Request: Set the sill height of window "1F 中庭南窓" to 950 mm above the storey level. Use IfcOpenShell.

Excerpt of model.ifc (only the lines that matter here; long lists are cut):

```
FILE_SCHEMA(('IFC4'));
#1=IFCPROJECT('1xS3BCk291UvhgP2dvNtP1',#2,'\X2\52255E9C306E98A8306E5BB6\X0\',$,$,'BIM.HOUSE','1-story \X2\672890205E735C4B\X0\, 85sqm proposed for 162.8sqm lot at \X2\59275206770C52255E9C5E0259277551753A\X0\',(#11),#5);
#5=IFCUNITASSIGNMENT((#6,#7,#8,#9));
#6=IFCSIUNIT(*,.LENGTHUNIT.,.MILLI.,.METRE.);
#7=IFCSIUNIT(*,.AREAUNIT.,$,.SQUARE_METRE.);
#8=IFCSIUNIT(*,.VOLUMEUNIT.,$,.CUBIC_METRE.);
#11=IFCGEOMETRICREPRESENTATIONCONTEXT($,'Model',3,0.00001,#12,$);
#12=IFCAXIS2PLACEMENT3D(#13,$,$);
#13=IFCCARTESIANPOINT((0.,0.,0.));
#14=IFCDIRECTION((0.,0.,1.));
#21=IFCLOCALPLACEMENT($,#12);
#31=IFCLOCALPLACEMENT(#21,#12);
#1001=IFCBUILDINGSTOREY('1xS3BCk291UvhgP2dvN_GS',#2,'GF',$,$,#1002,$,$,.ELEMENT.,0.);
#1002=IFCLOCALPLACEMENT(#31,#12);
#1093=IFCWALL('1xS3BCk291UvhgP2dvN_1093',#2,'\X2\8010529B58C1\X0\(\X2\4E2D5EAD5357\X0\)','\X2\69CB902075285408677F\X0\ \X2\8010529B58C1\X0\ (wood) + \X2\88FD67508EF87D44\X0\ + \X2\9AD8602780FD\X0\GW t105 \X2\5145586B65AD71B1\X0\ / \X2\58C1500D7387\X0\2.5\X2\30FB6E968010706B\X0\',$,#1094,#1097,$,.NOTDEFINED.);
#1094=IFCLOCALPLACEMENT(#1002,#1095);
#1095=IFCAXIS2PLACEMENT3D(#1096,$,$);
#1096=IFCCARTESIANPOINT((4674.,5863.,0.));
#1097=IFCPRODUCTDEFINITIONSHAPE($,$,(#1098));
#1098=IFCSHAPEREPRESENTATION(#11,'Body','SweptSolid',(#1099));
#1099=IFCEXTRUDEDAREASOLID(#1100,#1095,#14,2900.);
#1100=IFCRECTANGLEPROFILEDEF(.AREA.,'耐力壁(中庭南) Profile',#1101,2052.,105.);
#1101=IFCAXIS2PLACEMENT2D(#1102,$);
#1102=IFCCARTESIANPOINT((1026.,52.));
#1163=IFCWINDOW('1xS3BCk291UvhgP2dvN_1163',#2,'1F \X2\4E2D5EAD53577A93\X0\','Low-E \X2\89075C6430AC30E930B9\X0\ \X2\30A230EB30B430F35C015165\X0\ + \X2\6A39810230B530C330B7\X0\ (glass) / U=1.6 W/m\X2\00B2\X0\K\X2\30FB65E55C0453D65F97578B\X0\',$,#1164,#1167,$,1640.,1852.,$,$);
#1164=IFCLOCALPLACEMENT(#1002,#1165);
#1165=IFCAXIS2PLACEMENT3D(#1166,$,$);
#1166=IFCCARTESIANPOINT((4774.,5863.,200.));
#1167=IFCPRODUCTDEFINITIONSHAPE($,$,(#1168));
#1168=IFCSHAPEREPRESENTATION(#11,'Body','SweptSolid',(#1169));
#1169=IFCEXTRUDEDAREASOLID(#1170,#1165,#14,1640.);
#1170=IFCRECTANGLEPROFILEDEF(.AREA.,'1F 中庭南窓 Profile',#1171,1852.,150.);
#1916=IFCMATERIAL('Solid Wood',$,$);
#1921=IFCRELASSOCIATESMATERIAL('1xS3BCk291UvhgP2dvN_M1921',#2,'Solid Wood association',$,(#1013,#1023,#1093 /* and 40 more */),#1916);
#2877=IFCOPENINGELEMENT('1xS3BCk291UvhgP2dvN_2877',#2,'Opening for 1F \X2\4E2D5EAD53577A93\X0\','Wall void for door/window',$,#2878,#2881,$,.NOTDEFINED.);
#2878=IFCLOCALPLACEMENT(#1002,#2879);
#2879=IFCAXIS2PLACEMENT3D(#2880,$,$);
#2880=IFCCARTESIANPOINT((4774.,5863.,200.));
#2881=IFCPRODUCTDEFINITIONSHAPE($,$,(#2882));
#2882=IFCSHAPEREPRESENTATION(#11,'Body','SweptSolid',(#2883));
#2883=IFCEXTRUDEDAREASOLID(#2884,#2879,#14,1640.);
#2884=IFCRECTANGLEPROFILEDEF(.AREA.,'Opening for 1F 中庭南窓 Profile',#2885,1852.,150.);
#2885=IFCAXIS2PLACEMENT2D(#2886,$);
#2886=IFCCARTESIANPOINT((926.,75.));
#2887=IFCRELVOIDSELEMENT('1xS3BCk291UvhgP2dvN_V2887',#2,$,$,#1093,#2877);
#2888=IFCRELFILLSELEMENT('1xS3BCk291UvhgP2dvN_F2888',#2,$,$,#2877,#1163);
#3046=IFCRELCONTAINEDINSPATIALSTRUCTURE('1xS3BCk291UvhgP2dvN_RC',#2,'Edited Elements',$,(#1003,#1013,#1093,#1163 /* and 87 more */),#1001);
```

```python
import numpy as np
import ifcopenshell
import ifcopenshell.api.geometry
import ifcopenshell.geom
import ifcopenshell.util.element
import ifcopenshell.util.placement
import ifcopenshell.util.shape
import ifcopenshell.util.unit

model = ifcopenshell.open("model.ifc")
unit_scale = ifcopenshell.util.unit.calculate_unit_scale(model)

window = model.by_guid("1xS3BCk291UvhgP2dvN_1163")
opening = window.FillsVoids[0].RelatingOpeningElement
storey = ifcopenshell.util.element.get_container(window, ifc_class="IfcBuildingStorey")
level = ifcopenshell.util.placement.get_local_placement(storey.ObjectPlacement)[2, 3]

# The opening's origin need not be at the sill, so measure its lowest point.
shape = ifcopenshell.geom.create_shape(ifcopenshell.geom.settings(), opening)
bottom = ifcopenshell.util.shape.get_shape_bottom_elevation(shape, shape.geometry) / unit_scale
dz = level + 0.95 / unit_scale - bottom

shift = np.array([0.0, 0.0, dz])
# The window is not placed relative to its opening, so move both.
for product in (opening, window):
    matrix = ifcopenshell.util.placement.get_local_placement(product.ObjectPlacement)
    matrix[:3, 3] += shift
    ifcopenshell.api.geometry.edit_object_placement(model, product=product, matrix=matrix, is_si=False)

print(f"moved by {dz * unit_scale:+.3f} m")

model.write("model_v2.ifc")
```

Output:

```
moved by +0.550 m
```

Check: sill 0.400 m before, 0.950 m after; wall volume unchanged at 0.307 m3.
